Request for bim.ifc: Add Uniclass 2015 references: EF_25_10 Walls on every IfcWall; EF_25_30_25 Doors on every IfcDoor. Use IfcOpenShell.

First a look at what the model holds.

```python
import ifcopenshell

model = ifcopenshell.open("bim.ifc")
print(model.schema)
print("classifications:", [c.Name for c in model.by_type("IfcClassification")])
for ifc_class in ("IfcDoor", "IfcRoof", "IfcStair", "IfcWall", "IfcWindow"):
    print(ifc_class, len(model.by_type(ifc_class)))
```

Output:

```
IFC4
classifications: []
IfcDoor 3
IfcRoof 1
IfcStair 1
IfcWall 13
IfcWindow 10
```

```python
import ifcopenshell
import ifcopenshell.api.classification

model = ifcopenshell.open("bim.ifc")

system = ifcopenshell.api.classification.add_classification(model, classification="Uniclass 2015")

codes = {
    "IfcWall": ("EF_25_10", "Walls"),
    "IfcDoor": ("EF_25_30_25", "Doors"),
}
for ifc_class, (code, name) in codes.items():
    products = model.by_type(ifc_class)
    ifcopenshell.api.classification.add_reference(
        model, products=products, classification=system, identification=code, name=name
    )
    print(code, len(products))

model.write("bim-out.ifc")
```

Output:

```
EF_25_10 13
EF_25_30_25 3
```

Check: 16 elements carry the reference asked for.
